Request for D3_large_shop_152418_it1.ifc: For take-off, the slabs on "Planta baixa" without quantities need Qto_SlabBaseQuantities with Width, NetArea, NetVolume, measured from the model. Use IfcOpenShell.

First a look at what the model holds.

```python
import ifcopenshell
import ifcopenshell.util.element
import ifcopenshell.util.unit

model = ifcopenshell.open("D3_large_shop_152418_it1.ifc")
print(model.schema)
for unit_type in ("LENGTHUNIT", "AREAUNIT", "VOLUMEUNIT"):
    print(unit_type, ifcopenshell.util.unit.calculate_unit_scale(model, unit_type))
storey = next(s for s in model.by_type("IfcBuildingStorey") if s.Name == "Planta baixa")
slabs = [e for e in ifcopenshell.util.element.get_decomposition(storey) if e.is_a("IfcSlab")]
for e in sorted(slabs, key=lambda e: e.id()):
    print(e.id(), e.is_a(), e.Name, list(ifcopenshell.util.element.get_psets(e, qtos_only=True)), sep=" | ")
```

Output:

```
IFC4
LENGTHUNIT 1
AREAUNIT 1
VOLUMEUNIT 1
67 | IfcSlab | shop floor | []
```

```python
import ifcopenshell
import ifcopenshell.api.pset
import ifcopenshell.geom
import ifcopenshell.util.element
import ifcopenshell.util.shape
import ifcopenshell.util.unit

model = ifcopenshell.open("D3_large_shop_152418_it1.ifc")
unit_scale = ifcopenshell.util.unit.calculate_unit_scale(model)
area_scale = ifcopenshell.util.unit.calculate_unit_scale(model, "AREAUNIT")
volume_scale = ifcopenshell.util.unit.calculate_unit_scale(model, "VOLUMEUNIT")
settings = ifcopenshell.geom.settings()

storey = next(s for s in model.by_type("IfcBuildingStorey") if s.Name == "Planta baixa")
slabs = [e for e in ifcopenshell.util.element.get_decomposition(storey) if e.is_a("IfcSlab")]

for e in sorted(slabs, key=lambda e: e.id()):
    if ifcopenshell.util.element.get_psets(e, qtos_only=True, should_inherit=False):
        continue
    # Geometry comes back in metres, in the element's own axes.
    shape = ifcopenshell.geom.create_shape(settings, e)
    values = {
        "Width": ifcopenshell.util.shape.get_z(shape.geometry) / unit_scale,
        "NetArea": ifcopenshell.util.shape.get_footprint_area(shape.geometry) / area_scale,
        "NetVolume": ifcopenshell.util.shape.get_volume(shape.geometry) / volume_scale,
    }
    qto = ifcopenshell.api.pset.add_qto(model, product=e, name="Qto_SlabBaseQuantities")
    ifcopenshell.api.pset.edit_qto(model, qto=qto, properties=values)
    print(e.id(), {k: round(v, 3) for k, v in values.items()})

model.write("D3_large_shop_152418_it1-out.ifc")
```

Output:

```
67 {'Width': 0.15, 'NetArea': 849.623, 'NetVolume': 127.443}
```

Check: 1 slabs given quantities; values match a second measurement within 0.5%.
